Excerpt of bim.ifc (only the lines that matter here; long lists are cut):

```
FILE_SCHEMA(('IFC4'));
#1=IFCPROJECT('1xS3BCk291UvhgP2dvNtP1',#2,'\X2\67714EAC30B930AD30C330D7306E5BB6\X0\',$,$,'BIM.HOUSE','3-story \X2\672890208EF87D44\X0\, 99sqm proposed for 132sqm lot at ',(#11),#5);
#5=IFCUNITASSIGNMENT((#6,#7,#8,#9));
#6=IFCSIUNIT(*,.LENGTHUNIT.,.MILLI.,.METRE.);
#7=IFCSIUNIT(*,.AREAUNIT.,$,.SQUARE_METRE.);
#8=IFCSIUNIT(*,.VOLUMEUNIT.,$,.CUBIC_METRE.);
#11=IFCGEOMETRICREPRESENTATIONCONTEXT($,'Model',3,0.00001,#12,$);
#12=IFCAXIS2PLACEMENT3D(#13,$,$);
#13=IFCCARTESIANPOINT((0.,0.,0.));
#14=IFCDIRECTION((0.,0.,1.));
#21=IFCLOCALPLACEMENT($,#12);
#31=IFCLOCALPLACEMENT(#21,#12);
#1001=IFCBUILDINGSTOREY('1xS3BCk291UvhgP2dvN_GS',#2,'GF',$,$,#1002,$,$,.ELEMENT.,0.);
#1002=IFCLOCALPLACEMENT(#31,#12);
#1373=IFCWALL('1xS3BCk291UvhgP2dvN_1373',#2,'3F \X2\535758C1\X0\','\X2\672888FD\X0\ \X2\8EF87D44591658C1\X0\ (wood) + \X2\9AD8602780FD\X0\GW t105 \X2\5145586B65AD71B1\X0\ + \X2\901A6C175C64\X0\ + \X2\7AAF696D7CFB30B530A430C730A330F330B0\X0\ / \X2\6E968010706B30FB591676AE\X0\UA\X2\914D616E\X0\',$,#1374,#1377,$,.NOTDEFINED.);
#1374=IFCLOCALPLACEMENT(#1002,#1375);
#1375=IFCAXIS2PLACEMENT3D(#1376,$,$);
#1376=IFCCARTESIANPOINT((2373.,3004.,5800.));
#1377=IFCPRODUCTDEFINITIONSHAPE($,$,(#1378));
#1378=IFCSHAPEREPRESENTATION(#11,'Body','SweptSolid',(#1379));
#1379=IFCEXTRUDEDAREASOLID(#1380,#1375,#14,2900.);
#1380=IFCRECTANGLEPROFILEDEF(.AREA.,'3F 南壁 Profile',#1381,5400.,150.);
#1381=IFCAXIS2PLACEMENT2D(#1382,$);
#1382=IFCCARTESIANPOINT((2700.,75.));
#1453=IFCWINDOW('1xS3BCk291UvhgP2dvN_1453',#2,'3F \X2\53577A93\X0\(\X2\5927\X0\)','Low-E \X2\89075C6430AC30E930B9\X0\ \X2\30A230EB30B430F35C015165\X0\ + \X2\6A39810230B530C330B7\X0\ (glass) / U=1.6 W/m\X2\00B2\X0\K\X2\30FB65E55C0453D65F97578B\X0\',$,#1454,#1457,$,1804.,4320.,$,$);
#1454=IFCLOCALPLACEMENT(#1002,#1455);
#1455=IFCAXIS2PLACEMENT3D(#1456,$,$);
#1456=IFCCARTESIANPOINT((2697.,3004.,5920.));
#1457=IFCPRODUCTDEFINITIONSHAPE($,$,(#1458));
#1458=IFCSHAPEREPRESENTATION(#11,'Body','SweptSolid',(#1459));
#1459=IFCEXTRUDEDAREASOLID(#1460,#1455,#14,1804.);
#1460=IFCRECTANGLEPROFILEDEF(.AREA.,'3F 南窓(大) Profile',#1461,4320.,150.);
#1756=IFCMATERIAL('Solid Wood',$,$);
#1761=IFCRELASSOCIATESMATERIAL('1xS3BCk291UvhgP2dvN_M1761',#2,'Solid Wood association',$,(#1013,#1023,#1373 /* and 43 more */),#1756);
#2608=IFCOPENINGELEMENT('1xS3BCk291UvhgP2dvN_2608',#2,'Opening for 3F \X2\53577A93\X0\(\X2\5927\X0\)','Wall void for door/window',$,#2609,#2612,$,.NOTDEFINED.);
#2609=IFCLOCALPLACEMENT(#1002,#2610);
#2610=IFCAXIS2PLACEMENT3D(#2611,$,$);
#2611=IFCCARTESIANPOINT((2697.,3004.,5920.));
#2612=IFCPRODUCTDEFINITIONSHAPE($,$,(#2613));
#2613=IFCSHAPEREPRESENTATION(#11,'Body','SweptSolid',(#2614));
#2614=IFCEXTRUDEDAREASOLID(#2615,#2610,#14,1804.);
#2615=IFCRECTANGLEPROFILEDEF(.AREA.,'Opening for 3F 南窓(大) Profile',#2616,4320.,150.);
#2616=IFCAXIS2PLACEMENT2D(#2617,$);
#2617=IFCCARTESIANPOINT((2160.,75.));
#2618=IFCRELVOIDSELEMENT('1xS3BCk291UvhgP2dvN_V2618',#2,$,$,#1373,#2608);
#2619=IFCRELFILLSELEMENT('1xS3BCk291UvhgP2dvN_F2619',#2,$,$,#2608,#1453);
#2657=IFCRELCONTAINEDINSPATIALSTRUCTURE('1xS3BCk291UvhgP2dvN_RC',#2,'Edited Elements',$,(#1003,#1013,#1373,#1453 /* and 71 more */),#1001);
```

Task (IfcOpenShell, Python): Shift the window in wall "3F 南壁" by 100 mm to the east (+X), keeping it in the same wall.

```python
import ifcopenshell
import ifcopenshell.api.geometry
import ifcopenshell.util.placement
import ifcopenshell.util.unit

model = ifcopenshell.open("bim.ifc")
unit_scale = ifcopenshell.util.unit.calculate_unit_scale(model)

window = model.by_id(1453)
opening = window.FillsVoids[0].RelatingOpeningElement
wall = opening.VoidsElements[0].RelatingBuildingElement

wall_matrix = ifcopenshell.util.placement.get_local_placement(wall.ObjectPlacement)
shift = wall_matrix[:3, 0] * 0.1 / unit_scale
before = ifcopenshell.util.placement.get_local_placement(window.ObjectPlacement)[:3, 3].copy()

# The window is not placed relative to its opening, so move both.
for product in (opening, window):
    matrix = ifcopenshell.util.placement.get_local_placement(product.ObjectPlacement)
    matrix[:3, 3] += shift
    ifcopenshell.api.geometry.edit_object_placement(model, product=product, matrix=matrix, is_si=False)

after = ifcopenshell.util.placement.get_local_placement(window.ObjectPlacement)[:3, 3]
print("window moved by", (after - before).round(3) + 0.0)

model.write("bim_updated.ifc")
```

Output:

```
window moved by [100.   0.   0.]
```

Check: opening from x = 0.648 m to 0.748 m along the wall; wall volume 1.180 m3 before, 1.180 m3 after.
